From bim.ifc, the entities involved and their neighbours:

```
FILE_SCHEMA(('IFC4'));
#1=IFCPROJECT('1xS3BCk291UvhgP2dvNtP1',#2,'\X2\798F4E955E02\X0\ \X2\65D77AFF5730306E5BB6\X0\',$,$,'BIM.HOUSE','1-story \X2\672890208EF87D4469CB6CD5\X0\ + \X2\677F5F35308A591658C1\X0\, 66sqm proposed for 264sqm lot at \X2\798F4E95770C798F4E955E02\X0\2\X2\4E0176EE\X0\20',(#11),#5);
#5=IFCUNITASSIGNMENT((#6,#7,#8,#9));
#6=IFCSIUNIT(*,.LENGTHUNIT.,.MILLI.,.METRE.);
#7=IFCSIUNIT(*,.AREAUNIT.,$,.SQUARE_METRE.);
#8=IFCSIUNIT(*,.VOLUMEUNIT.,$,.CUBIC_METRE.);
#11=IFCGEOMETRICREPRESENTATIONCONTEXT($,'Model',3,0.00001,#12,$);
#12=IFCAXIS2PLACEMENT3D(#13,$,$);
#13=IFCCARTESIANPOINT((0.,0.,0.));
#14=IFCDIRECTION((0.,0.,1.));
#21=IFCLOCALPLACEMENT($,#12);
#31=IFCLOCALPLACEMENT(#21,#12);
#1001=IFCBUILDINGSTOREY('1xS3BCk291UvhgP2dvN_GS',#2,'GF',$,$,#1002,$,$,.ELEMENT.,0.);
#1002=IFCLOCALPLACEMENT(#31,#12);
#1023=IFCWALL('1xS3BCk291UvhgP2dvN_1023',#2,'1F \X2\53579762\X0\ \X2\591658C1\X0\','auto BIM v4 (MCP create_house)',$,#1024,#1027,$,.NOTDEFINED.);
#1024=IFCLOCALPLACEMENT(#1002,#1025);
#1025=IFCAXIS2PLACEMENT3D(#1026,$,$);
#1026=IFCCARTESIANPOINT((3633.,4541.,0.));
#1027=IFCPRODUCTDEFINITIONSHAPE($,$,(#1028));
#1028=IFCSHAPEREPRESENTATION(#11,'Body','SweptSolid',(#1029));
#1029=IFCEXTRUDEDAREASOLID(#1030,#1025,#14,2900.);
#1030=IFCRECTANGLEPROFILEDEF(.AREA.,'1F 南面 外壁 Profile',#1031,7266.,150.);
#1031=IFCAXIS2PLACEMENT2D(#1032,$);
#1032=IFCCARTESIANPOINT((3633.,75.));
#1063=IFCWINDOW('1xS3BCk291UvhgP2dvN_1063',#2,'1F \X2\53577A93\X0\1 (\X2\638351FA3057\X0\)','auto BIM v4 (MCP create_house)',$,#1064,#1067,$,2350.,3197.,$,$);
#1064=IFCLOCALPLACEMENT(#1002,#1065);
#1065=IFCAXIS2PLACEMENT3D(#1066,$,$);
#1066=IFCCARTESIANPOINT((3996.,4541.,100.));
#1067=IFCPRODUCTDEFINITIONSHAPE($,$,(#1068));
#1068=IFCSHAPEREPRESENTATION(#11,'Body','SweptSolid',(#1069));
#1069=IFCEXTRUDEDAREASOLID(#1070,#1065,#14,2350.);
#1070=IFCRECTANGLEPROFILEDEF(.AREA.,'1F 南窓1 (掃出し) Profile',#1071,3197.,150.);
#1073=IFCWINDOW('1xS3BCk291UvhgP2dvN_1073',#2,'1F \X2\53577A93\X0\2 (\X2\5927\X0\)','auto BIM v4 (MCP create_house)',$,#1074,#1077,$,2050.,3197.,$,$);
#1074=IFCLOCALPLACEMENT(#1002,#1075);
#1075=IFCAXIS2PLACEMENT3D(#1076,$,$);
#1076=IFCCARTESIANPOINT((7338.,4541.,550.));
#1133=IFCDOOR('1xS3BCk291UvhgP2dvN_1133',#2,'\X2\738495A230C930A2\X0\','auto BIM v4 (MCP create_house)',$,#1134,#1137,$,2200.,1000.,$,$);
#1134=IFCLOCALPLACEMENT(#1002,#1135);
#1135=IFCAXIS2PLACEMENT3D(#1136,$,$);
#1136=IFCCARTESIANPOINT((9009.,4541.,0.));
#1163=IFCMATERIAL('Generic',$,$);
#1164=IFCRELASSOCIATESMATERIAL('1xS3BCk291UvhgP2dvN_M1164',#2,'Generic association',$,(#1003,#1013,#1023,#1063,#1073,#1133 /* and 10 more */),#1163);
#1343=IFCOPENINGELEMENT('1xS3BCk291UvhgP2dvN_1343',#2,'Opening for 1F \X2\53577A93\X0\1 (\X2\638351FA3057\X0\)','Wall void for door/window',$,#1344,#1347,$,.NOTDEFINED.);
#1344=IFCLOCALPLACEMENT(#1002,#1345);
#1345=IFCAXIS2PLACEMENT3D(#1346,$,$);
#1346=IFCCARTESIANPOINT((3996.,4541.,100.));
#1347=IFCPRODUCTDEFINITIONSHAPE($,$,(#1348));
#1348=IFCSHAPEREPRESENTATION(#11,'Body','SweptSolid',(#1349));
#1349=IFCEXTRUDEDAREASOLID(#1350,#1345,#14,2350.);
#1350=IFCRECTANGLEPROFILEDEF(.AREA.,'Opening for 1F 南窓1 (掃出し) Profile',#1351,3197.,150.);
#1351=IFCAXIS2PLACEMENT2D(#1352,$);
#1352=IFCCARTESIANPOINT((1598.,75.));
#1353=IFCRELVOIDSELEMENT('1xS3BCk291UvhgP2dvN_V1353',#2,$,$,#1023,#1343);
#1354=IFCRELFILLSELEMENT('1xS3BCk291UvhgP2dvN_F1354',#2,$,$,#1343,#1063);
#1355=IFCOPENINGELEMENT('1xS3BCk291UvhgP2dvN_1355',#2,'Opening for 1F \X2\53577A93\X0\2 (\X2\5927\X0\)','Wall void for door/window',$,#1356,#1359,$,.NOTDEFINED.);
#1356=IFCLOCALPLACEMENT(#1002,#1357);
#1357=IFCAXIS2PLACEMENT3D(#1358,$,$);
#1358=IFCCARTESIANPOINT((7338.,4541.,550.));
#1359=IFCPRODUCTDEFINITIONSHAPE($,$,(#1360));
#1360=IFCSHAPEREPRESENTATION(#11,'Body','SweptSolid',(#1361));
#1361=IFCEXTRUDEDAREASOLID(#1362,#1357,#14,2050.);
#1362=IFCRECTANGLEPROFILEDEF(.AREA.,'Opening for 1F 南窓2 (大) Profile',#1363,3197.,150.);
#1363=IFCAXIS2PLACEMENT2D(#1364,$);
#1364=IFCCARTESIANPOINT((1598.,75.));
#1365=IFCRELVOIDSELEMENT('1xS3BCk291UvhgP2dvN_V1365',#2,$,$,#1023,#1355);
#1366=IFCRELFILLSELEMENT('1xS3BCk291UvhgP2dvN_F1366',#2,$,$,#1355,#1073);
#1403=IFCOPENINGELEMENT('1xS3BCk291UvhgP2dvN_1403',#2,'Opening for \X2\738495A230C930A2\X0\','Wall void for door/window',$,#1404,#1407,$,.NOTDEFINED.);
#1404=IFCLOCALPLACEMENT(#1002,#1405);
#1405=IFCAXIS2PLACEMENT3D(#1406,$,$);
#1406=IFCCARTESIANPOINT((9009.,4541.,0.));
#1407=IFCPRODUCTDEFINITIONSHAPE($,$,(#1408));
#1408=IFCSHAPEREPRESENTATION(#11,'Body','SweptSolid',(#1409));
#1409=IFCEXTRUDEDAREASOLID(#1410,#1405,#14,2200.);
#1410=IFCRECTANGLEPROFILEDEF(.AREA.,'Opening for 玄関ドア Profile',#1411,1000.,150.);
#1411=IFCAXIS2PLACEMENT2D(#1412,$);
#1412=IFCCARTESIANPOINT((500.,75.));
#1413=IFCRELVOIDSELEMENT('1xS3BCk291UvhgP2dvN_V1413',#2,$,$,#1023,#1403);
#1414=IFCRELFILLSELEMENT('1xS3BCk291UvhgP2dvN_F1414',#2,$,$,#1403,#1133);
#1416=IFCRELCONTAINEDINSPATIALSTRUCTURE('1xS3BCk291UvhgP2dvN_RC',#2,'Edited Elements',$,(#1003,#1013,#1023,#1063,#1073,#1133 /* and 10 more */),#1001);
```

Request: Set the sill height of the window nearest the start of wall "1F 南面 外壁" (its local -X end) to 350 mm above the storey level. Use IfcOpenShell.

```python
import numpy as np
import ifcopenshell
import ifcopenshell.api.geometry
import ifcopenshell.geom
import ifcopenshell.util.element
import ifcopenshell.util.placement
import ifcopenshell.util.shape
import ifcopenshell.util.unit

model = ifcopenshell.open("bim.ifc")
unit_scale = ifcopenshell.util.unit.calculate_unit_scale(model)

window = model.by_guid("1xS3BCk291UvhgP2dvN_1063")
opening = window.FillsVoids[0].RelatingOpeningElement
storey = ifcopenshell.util.element.get_container(window, ifc_class="IfcBuildingStorey")
level = ifcopenshell.util.placement.get_local_placement(storey.ObjectPlacement)[2, 3]

# The opening's origin need not be at the sill, so measure its lowest point.
shape = ifcopenshell.geom.create_shape(ifcopenshell.geom.settings(), opening)
bottom = ifcopenshell.util.shape.get_shape_bottom_elevation(shape, shape.geometry) / unit_scale
dz = level + 0.35 / unit_scale - bottom

shift = np.array([0.0, 0.0, dz])
# The window is not placed relative to its opening, so move both.
for product in (opening, window):
    matrix = ifcopenshell.util.placement.get_local_placement(product.ObjectPlacement)
    matrix[:3, 3] += shift
    ifcopenshell.api.geometry.edit_object_placement(model, product=product, matrix=matrix, is_si=False)

print(f"moved by {dz * unit_scale:+.3f} m")

model.write("bim_edited.ifc")
```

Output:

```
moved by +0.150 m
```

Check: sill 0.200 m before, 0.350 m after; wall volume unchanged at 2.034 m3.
